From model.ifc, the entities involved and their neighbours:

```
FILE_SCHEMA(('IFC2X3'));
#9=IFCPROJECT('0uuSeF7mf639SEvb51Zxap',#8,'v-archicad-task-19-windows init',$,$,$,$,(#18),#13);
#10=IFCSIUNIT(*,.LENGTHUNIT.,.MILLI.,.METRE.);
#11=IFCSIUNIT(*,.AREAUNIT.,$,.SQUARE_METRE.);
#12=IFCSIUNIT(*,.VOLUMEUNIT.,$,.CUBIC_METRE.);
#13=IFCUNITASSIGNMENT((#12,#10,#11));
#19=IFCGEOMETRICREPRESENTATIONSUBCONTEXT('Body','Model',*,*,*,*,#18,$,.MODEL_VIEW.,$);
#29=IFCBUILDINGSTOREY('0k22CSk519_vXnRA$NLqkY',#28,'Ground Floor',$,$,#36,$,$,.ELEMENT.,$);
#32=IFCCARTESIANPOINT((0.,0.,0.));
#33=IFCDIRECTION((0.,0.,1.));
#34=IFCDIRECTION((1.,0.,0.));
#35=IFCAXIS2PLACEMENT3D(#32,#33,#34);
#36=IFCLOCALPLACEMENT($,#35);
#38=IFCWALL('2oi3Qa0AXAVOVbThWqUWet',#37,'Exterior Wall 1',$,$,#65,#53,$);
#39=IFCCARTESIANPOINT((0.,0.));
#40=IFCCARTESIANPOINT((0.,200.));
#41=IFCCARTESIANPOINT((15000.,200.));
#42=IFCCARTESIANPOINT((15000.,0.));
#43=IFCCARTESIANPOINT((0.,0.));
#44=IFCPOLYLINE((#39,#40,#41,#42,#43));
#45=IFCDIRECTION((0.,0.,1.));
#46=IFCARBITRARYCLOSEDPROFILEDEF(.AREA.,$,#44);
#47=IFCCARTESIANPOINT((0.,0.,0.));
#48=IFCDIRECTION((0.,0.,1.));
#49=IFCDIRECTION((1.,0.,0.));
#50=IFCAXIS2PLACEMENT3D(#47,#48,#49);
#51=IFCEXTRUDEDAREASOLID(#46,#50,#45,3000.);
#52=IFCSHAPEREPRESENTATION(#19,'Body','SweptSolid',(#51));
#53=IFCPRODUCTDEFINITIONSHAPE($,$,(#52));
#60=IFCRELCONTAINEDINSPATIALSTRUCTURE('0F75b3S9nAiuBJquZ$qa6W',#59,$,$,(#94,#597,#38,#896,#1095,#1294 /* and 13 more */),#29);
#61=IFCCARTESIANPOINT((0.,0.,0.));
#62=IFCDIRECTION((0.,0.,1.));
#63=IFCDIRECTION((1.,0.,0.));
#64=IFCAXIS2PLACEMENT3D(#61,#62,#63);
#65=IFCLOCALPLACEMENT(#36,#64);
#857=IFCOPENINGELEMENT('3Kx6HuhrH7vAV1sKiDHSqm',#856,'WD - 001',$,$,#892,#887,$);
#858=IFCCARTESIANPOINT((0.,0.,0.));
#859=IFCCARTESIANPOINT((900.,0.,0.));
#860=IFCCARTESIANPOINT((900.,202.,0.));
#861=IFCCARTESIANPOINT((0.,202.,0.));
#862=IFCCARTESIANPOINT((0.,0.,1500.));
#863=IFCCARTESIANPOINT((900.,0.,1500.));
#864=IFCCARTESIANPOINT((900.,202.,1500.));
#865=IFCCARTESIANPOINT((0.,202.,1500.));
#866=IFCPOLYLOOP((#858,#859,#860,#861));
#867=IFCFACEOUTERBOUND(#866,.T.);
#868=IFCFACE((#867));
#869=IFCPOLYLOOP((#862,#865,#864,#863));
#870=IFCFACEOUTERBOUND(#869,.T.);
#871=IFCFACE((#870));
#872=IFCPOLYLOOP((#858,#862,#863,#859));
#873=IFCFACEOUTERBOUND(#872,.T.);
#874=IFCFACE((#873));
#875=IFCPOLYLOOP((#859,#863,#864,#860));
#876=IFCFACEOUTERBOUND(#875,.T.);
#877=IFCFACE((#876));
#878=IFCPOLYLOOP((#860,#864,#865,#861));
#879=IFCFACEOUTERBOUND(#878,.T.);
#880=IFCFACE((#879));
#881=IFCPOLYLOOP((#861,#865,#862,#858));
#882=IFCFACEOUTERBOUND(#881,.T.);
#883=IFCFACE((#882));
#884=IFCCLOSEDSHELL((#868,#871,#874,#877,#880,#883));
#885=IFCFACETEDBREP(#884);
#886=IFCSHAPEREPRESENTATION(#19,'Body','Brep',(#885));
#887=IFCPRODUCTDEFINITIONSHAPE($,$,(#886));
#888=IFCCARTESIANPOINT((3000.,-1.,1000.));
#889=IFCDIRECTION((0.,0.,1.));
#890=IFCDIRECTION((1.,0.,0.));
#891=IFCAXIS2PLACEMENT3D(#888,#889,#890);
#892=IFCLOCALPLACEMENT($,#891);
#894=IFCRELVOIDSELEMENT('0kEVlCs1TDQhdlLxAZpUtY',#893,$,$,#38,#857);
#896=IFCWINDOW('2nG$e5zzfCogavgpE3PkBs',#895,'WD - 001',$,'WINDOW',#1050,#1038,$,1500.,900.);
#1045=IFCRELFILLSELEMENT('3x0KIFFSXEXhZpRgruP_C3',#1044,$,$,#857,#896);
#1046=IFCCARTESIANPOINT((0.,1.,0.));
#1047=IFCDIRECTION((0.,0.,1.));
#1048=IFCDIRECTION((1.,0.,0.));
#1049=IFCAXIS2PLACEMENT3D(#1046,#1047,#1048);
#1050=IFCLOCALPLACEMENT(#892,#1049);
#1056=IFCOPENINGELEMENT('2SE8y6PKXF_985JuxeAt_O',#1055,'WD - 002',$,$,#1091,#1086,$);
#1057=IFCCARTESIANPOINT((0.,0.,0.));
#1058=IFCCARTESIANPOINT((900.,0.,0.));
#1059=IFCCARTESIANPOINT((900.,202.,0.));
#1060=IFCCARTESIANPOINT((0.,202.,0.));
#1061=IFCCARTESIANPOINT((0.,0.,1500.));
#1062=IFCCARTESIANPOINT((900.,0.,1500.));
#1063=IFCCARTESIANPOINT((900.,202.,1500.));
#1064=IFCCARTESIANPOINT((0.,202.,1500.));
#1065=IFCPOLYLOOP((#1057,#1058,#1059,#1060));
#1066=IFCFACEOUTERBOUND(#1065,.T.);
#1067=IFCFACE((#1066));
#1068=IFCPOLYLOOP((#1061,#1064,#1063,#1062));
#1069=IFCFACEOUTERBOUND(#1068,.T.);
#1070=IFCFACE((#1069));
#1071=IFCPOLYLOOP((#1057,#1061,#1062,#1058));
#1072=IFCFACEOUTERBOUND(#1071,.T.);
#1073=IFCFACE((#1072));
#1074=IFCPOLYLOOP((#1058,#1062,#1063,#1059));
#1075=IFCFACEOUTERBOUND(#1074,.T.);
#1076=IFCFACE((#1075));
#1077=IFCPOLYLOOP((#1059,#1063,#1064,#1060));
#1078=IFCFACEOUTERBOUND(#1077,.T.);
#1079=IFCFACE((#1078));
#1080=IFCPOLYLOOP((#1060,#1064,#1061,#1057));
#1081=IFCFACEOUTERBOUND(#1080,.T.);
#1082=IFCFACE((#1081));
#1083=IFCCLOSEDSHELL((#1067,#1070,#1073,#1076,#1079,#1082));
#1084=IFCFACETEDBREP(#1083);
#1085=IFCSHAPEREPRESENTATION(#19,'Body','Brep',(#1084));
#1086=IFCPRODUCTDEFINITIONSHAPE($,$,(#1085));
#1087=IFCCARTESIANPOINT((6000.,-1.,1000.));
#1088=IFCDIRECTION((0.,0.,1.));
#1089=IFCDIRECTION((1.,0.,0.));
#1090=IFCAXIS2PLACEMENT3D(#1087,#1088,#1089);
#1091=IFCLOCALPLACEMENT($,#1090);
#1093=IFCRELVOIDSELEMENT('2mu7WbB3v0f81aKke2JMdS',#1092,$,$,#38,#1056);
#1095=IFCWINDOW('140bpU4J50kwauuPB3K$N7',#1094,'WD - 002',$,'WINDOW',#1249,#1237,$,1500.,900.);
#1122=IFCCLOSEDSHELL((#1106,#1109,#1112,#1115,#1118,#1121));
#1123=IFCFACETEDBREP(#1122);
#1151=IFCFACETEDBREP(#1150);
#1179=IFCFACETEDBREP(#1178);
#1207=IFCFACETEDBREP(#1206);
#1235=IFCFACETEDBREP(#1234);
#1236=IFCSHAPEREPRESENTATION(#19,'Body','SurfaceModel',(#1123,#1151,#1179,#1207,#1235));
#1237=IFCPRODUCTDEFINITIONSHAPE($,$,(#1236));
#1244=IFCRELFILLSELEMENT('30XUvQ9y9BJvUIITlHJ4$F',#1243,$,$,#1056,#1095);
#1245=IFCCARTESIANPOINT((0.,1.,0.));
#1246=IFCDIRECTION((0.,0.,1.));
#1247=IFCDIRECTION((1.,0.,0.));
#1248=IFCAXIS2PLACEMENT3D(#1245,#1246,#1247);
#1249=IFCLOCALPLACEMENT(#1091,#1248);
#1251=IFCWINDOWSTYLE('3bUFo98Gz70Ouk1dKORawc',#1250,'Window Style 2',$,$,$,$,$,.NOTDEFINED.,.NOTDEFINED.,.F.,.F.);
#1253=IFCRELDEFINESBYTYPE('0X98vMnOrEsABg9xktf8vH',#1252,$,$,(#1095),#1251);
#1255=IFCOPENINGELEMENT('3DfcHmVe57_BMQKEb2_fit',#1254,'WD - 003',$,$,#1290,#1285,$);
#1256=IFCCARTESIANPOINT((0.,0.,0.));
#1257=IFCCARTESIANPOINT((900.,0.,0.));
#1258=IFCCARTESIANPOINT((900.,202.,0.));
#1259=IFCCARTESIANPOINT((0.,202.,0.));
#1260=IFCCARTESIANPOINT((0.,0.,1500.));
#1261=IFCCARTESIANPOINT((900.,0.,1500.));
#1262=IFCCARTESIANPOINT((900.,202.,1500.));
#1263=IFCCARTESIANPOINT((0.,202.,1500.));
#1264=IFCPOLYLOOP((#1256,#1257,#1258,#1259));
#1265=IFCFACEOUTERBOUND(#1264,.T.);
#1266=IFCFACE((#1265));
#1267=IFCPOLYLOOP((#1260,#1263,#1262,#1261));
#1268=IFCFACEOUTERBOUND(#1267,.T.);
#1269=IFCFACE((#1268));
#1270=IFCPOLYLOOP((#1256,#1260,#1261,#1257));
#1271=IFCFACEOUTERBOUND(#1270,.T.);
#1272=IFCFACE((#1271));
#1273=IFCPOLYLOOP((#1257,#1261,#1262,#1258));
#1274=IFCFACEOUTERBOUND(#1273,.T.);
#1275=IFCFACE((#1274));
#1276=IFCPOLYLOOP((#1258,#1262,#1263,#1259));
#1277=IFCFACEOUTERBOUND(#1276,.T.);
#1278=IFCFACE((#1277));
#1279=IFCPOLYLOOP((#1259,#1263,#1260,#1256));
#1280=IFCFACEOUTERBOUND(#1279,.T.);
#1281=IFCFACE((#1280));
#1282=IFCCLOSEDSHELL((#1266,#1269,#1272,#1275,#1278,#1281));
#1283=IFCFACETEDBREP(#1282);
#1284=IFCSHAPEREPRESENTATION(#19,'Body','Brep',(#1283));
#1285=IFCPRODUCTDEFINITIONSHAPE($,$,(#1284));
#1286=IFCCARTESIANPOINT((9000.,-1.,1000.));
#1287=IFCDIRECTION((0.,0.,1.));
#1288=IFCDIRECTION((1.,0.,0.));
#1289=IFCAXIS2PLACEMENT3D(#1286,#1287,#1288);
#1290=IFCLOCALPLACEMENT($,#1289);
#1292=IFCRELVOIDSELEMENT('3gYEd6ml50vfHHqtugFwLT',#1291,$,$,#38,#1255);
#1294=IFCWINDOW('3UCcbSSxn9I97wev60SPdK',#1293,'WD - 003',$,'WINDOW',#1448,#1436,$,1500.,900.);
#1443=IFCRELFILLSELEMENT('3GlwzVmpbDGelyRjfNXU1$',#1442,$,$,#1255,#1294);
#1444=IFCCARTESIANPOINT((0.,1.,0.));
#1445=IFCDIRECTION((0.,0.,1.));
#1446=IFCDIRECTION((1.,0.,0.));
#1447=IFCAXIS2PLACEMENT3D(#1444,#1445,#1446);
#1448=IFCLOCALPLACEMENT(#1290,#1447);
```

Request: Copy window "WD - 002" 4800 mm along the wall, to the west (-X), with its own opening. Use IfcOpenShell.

```python
import ifcopenshell
import ifcopenshell.api.feature
import ifcopenshell.api.geometry
import ifcopenshell.api.root
import ifcopenshell.geom
import ifcopenshell.util.element
import ifcopenshell.util.placement
import ifcopenshell.util.shape
import ifcopenshell.util.unit

model = ifcopenshell.open("model.ifc")
unit_scale = ifcopenshell.util.unit.calculate_unit_scale(model)
settings = ifcopenshell.geom.settings()


def volume(element):
    """Net volume in cubic metres, openings subtracted."""
    shape = ifcopenshell.geom.create_shape(settings, element)
    return ifcopenshell.util.shape.get_volume(shape.geometry)


window = model.by_id(1095)
opening = window.FillsVoids[0].RelatingOpeningElement
wall = opening.VoidsElements[0].RelatingBuildingElement
before = volume(wall)
shift = ifcopenshell.util.placement.get_local_placement(wall.ObjectPlacement)[:3, 0] * -4.8 / unit_scale

# copy_class copies the void relationship, type, container and properties, but no geometry.
new_opening = ifcopenshell.api.root.copy_class(model, product=opening)
new_opening.Representation = ifcopenshell.util.element.copy_deep(
    model, opening.Representation, exclude=["IfcGeometricRepresentationContext", "IfcRepresentationMap"]
)
new_window = ifcopenshell.api.root.copy_class(model, product=window)
new_window.Representation = ifcopenshell.util.element.copy_deep(
    model, window.Representation, exclude=["IfcGeometricRepresentationContext", "IfcRepresentationMap"]
)
fills = ifcopenshell.api.feature.add_filling(model, opening=new_opening, element=new_window)
fills.OwnerHistory = new_window.OwnerHistory  # required in IFC2X3

for old, new in ((opening, new_opening), (window, new_window)):
    matrix = ifcopenshell.util.placement.get_local_placement(old.ObjectPlacement)
    matrix[:3, 3] += shift
    ifcopenshell.api.geometry.edit_object_placement(model, product=new, matrix=matrix, is_si=False)

after = volume(wall)

print(f"wall volume {before:.3f} -> {after:.3f} m3")

model.write("model_edited.ifc")
```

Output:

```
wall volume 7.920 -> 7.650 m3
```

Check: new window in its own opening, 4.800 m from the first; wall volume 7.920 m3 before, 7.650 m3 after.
